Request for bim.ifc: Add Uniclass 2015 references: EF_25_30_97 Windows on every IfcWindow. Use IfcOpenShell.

First a look at what the model holds.

```python
import ifcopenshell

model = ifcopenshell.open("bim.ifc")
print(model.schema)
print("classifications:", [c.Name for c in model.by_type("IfcClassification")])
for ifc_class in ("IfcDoor", "IfcRoof", "IfcStair", "IfcWall", "IfcWindow"):
    print(ifc_class, len(model.by_type(ifc_class)))
```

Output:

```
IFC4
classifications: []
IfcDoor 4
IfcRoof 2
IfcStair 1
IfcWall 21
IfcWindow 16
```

```python
import ifcopenshell
import ifcopenshell.api.classification

model = ifcopenshell.open("bim.ifc")

system = ifcopenshell.api.classification.add_classification(model, classification="Uniclass 2015")

codes = {
    "IfcWindow": ("EF_25_30_97", "Windows"),
}
for ifc_class, (code, name) in codes.items():
    products = model.by_type(ifc_class)
    ifcopenshell.api.classification.add_reference(
        model, products=products, classification=system, identification=code, name=name
    )
    print(code, len(products))

model.write("bim_edited.ifc")
```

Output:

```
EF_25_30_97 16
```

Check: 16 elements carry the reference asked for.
